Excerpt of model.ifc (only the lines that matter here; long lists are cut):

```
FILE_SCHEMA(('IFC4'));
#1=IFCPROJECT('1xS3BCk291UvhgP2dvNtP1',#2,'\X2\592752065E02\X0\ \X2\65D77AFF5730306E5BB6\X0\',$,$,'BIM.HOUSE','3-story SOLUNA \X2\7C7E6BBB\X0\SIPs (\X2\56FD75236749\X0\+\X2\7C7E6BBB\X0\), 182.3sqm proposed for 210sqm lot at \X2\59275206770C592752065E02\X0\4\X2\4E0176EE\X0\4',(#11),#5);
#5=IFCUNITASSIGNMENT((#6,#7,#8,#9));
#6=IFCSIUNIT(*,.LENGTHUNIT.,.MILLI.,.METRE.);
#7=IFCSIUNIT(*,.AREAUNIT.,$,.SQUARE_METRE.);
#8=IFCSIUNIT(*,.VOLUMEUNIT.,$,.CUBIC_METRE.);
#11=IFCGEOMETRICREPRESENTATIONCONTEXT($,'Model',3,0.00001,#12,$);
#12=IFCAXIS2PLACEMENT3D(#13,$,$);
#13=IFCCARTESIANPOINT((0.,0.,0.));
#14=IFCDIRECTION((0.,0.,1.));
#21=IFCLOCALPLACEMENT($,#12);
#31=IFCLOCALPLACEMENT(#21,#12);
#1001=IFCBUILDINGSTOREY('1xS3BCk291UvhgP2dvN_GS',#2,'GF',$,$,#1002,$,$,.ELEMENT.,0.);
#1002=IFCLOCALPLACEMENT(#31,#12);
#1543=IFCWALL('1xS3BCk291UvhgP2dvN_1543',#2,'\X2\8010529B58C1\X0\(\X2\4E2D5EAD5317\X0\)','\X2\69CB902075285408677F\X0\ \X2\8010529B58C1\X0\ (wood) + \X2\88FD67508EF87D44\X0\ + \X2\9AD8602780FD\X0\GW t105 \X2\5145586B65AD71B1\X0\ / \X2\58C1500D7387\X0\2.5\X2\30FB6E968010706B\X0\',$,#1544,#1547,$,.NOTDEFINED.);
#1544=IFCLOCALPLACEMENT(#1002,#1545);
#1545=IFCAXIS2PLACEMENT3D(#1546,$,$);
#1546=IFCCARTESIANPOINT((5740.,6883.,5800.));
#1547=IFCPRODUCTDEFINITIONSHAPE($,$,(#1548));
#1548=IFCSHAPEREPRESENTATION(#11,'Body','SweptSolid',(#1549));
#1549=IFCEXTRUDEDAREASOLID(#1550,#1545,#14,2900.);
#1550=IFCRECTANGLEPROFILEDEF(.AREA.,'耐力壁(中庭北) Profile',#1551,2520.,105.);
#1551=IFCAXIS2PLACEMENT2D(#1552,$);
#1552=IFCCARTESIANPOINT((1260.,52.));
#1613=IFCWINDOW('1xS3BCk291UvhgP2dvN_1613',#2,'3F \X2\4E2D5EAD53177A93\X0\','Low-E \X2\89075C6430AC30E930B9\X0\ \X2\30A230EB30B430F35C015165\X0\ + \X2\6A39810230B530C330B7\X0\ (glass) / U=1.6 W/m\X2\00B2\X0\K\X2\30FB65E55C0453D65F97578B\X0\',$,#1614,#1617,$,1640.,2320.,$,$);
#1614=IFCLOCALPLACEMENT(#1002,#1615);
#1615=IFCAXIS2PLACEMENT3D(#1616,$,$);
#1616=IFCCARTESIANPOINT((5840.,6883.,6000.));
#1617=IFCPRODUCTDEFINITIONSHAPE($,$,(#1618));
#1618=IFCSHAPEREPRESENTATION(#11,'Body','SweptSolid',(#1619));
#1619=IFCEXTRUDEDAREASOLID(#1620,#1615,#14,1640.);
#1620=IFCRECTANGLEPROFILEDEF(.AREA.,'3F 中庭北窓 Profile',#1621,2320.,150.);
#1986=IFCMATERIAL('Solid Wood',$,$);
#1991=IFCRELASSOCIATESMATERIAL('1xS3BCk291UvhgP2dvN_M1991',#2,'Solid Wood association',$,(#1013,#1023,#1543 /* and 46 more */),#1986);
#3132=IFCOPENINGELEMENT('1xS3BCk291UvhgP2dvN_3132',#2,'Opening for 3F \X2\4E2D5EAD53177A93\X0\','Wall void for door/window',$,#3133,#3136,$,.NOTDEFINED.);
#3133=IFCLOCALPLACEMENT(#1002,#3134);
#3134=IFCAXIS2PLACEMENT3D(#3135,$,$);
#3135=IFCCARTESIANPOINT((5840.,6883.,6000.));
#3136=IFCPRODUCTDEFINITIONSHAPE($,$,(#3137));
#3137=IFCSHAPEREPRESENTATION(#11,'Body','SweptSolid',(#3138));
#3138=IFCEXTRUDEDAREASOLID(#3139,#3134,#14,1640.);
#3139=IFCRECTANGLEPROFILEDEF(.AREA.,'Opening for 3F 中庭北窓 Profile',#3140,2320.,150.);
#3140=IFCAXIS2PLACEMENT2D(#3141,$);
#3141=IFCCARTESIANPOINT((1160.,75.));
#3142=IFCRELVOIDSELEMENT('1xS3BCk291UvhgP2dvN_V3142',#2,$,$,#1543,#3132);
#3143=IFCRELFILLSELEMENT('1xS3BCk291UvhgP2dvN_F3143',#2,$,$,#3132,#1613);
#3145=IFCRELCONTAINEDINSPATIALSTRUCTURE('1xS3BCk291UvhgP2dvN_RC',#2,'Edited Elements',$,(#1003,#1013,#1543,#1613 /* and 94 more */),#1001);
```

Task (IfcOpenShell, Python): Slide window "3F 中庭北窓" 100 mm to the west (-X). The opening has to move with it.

```python
import ifcopenshell
import ifcopenshell.api.geometry
import ifcopenshell.util.placement

model = ifcopenshell.open("model.ifc")

window = model.by_guid("1xS3BCk291UvhgP2dvN_1613")
opening = window.FillsVoids[0].RelatingOpeningElement
wall = opening.VoidsElements[0].RelatingBuildingElement

wall_matrix = ifcopenshell.util.placement.get_local_placement(wall.ObjectPlacement)
shift = wall_matrix[:3, 0] * -100.0
before = ifcopenshell.util.placement.get_local_placement(window.ObjectPlacement)[:3, 3].copy()

# The window is not placed relative to its opening, so move both.
for product in (opening, window):
    matrix = ifcopenshell.util.placement.get_local_placement(product.ObjectPlacement)
    matrix[:3, 3] += shift
    ifcopenshell.api.geometry.edit_object_placement(model, product=product, matrix=matrix, is_si=False)

after = ifcopenshell.util.placement.get_local_placement(window.ObjectPlacement)[:3, 3]
print("window moved by", (after - before).round(3) + 0.0)

model.write("model_updated.ifc")
```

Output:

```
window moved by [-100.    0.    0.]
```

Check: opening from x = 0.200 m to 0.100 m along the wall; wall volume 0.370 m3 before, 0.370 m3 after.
